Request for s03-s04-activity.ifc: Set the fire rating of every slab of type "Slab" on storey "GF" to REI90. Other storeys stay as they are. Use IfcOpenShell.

First a look at what the model holds.

```python
import ifcopenshell
import ifcopenshell.util.element

model = ifcopenshell.open("s03-s04-activity.ifc")
print(model.schema)
storey = next(s for s in model.by_type("IfcBuildingStorey") if s.Name == "GF")
slabs = [e for e in ifcopenshell.util.element.get_decomposition(storey) if e.is_a("IfcSlab")]
seen = {}
for e in slabs:
    element_type = ifcopenshell.util.element.get_type(e)
    key = (element_type.Name if element_type != e and element_type else None, ifcopenshell.util.element.get_pset(e, "Pset_SlabCommon", "FireRating"))
    seen[key] = seen.get(key, 0) + 1
for (name, value), count in sorted(seen.items(), key=str):
    print(count, "x", name, "|", value)
```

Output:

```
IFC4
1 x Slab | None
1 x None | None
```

```python
import ifcopenshell
import ifcopenshell.api.pset
import ifcopenshell.util.element

model = ifcopenshell.open("s03-s04-activity.ifc")

storey = next(s for s in model.by_type("IfcBuildingStorey") if s.Name == "GF")
slabs = [e for e in ifcopenshell.util.element.get_decomposition(storey) if e.is_a("IfcSlab")]

count = 0
for e in slabs:
    element_type = ifcopenshell.util.element.get_type(e)
    if element_type in (None, e) or element_type.Name != "Slab":
        continue
    # add_pset returns the element's existing set when there is one.
    pset = ifcopenshell.api.pset.add_pset(model, product=e, name="Pset_SlabCommon")
    ifcopenshell.api.pset.edit_pset(model, pset=pset, properties={"FireRating": "REI90"})
    count += 1

print(count, "slabs updated")

model.write("s03-s04-activity_updated.ifc")
```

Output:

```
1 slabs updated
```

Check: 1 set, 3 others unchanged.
